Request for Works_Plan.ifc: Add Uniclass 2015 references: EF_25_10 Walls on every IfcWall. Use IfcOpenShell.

First a look at what the model holds.

```python
import ifcopenshell

model = ifcopenshell.open("Works_Plan.ifc")
print(model.schema)
print("classifications:", [c.Name for c in model.by_type("IfcClassification")])
for ifc_class in ("IfcDoor", "IfcRoof", "IfcStair", "IfcWall", "IfcWindow"):
    print(ifc_class, len(model.by_type(ifc_class)))
```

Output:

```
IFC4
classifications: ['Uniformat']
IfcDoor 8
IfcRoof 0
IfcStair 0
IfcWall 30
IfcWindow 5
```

```python
import ifcopenshell
import ifcopenshell.api.classification

model = ifcopenshell.open("Works_Plan.ifc")

system = ifcopenshell.api.classification.add_classification(model, classification="Uniclass 2015")

codes = {
    "IfcWall": ("EF_25_10", "Walls"),
}
for ifc_class, (code, name) in codes.items():
    products = model.by_type(ifc_class)
    ifcopenshell.api.classification.add_reference(
        model, products=products, classification=system, identification=code, name=name
    )
    print(code, len(products))

model.write("Works_Plan-out.ifc")
```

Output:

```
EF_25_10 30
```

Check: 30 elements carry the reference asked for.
